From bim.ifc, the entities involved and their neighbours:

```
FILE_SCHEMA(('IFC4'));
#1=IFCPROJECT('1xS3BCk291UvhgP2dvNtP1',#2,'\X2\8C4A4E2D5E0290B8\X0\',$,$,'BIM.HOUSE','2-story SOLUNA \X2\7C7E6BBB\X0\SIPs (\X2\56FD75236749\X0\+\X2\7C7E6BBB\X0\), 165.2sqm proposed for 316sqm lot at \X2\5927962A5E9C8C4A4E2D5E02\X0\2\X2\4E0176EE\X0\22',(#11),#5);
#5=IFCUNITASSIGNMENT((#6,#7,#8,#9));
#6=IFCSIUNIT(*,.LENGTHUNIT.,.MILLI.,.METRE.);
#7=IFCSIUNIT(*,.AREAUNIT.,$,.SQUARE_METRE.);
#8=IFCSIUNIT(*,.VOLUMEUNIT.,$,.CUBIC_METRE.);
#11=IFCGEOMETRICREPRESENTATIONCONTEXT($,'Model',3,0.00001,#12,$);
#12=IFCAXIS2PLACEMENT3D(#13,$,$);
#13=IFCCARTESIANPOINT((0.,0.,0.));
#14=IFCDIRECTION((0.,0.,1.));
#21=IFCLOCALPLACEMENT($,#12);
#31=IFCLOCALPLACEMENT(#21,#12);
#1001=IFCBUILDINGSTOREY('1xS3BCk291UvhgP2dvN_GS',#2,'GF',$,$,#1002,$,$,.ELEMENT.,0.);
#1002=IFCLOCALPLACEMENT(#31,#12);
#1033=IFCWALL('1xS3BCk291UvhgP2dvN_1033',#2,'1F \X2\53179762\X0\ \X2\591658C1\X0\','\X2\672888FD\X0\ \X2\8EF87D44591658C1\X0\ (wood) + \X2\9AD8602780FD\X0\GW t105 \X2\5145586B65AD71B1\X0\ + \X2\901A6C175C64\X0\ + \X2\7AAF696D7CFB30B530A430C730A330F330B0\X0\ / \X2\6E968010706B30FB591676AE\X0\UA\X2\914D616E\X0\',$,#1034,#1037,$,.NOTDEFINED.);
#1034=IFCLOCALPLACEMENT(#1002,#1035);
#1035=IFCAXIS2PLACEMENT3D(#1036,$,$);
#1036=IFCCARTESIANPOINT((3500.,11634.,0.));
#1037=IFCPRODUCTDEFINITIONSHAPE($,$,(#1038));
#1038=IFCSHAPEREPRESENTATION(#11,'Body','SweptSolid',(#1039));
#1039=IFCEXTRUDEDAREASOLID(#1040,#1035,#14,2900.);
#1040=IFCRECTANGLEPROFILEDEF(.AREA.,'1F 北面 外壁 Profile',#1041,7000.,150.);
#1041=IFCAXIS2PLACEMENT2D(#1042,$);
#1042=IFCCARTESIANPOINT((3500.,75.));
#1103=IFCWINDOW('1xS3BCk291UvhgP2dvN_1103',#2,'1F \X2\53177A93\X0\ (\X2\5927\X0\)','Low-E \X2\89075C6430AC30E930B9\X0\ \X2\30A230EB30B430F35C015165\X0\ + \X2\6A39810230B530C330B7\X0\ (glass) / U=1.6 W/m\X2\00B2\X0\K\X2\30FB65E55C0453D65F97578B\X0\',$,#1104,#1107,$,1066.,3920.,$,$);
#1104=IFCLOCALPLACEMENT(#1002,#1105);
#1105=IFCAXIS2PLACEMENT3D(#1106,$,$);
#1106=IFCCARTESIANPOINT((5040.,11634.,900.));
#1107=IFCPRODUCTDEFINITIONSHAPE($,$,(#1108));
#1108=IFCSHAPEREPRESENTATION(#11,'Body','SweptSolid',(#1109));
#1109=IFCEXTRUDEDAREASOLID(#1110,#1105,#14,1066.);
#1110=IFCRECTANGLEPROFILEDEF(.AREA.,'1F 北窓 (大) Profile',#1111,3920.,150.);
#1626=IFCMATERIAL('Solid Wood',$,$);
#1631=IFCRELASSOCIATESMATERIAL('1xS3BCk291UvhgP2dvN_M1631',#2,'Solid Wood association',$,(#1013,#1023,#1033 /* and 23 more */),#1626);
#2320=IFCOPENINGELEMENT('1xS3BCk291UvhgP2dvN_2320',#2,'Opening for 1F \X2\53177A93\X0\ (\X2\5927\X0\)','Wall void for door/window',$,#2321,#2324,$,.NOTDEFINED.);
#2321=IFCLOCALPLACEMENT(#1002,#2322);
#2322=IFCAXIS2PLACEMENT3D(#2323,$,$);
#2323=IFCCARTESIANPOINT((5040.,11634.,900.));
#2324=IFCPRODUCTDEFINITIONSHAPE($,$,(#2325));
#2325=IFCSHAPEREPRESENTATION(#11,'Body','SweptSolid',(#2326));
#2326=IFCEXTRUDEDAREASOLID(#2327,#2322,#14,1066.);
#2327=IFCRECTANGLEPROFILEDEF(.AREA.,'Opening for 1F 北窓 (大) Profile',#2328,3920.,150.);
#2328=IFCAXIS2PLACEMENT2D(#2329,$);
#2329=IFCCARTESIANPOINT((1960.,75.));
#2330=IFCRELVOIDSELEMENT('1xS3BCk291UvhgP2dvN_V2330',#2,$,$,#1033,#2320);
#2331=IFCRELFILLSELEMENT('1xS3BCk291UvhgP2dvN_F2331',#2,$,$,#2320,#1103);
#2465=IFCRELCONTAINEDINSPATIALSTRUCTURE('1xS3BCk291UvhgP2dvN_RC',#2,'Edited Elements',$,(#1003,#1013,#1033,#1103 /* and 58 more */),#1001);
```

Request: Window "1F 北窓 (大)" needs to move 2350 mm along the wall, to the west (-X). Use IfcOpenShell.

```python
import ifcopenshell
import ifcopenshell.api.geometry
import ifcopenshell.util.placement
import ifcopenshell.util.unit

model = ifcopenshell.open("bim.ifc")
unit_scale = ifcopenshell.util.unit.calculate_unit_scale(model)

window = model.by_guid("1xS3BCk291UvhgP2dvN_1103")
opening = window.FillsVoids[0].RelatingOpeningElement
wall = opening.VoidsElements[0].RelatingBuildingElement

wall_matrix = ifcopenshell.util.placement.get_local_placement(wall.ObjectPlacement)
shift = wall_matrix[:3, 0] * -2.35 / unit_scale
before = ifcopenshell.util.placement.get_local_placement(window.ObjectPlacement)[:3, 3].copy()

# The window is not placed relative to its opening, so move both.
for product in (opening, window):
    matrix = ifcopenshell.util.placement.get_local_placement(product.ObjectPlacement)
    matrix[:3, 3] += shift
    ifcopenshell.api.geometry.edit_object_placement(model, product=product, matrix=matrix, is_si=False)

after = ifcopenshell.util.placement.get_local_placement(window.ObjectPlacement)[:3, 3]
print("window moved by", (after - before).round(3) + 0.0)

model.write("bim_edited.ifc")
```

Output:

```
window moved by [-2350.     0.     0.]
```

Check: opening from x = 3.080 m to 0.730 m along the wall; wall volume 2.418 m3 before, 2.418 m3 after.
